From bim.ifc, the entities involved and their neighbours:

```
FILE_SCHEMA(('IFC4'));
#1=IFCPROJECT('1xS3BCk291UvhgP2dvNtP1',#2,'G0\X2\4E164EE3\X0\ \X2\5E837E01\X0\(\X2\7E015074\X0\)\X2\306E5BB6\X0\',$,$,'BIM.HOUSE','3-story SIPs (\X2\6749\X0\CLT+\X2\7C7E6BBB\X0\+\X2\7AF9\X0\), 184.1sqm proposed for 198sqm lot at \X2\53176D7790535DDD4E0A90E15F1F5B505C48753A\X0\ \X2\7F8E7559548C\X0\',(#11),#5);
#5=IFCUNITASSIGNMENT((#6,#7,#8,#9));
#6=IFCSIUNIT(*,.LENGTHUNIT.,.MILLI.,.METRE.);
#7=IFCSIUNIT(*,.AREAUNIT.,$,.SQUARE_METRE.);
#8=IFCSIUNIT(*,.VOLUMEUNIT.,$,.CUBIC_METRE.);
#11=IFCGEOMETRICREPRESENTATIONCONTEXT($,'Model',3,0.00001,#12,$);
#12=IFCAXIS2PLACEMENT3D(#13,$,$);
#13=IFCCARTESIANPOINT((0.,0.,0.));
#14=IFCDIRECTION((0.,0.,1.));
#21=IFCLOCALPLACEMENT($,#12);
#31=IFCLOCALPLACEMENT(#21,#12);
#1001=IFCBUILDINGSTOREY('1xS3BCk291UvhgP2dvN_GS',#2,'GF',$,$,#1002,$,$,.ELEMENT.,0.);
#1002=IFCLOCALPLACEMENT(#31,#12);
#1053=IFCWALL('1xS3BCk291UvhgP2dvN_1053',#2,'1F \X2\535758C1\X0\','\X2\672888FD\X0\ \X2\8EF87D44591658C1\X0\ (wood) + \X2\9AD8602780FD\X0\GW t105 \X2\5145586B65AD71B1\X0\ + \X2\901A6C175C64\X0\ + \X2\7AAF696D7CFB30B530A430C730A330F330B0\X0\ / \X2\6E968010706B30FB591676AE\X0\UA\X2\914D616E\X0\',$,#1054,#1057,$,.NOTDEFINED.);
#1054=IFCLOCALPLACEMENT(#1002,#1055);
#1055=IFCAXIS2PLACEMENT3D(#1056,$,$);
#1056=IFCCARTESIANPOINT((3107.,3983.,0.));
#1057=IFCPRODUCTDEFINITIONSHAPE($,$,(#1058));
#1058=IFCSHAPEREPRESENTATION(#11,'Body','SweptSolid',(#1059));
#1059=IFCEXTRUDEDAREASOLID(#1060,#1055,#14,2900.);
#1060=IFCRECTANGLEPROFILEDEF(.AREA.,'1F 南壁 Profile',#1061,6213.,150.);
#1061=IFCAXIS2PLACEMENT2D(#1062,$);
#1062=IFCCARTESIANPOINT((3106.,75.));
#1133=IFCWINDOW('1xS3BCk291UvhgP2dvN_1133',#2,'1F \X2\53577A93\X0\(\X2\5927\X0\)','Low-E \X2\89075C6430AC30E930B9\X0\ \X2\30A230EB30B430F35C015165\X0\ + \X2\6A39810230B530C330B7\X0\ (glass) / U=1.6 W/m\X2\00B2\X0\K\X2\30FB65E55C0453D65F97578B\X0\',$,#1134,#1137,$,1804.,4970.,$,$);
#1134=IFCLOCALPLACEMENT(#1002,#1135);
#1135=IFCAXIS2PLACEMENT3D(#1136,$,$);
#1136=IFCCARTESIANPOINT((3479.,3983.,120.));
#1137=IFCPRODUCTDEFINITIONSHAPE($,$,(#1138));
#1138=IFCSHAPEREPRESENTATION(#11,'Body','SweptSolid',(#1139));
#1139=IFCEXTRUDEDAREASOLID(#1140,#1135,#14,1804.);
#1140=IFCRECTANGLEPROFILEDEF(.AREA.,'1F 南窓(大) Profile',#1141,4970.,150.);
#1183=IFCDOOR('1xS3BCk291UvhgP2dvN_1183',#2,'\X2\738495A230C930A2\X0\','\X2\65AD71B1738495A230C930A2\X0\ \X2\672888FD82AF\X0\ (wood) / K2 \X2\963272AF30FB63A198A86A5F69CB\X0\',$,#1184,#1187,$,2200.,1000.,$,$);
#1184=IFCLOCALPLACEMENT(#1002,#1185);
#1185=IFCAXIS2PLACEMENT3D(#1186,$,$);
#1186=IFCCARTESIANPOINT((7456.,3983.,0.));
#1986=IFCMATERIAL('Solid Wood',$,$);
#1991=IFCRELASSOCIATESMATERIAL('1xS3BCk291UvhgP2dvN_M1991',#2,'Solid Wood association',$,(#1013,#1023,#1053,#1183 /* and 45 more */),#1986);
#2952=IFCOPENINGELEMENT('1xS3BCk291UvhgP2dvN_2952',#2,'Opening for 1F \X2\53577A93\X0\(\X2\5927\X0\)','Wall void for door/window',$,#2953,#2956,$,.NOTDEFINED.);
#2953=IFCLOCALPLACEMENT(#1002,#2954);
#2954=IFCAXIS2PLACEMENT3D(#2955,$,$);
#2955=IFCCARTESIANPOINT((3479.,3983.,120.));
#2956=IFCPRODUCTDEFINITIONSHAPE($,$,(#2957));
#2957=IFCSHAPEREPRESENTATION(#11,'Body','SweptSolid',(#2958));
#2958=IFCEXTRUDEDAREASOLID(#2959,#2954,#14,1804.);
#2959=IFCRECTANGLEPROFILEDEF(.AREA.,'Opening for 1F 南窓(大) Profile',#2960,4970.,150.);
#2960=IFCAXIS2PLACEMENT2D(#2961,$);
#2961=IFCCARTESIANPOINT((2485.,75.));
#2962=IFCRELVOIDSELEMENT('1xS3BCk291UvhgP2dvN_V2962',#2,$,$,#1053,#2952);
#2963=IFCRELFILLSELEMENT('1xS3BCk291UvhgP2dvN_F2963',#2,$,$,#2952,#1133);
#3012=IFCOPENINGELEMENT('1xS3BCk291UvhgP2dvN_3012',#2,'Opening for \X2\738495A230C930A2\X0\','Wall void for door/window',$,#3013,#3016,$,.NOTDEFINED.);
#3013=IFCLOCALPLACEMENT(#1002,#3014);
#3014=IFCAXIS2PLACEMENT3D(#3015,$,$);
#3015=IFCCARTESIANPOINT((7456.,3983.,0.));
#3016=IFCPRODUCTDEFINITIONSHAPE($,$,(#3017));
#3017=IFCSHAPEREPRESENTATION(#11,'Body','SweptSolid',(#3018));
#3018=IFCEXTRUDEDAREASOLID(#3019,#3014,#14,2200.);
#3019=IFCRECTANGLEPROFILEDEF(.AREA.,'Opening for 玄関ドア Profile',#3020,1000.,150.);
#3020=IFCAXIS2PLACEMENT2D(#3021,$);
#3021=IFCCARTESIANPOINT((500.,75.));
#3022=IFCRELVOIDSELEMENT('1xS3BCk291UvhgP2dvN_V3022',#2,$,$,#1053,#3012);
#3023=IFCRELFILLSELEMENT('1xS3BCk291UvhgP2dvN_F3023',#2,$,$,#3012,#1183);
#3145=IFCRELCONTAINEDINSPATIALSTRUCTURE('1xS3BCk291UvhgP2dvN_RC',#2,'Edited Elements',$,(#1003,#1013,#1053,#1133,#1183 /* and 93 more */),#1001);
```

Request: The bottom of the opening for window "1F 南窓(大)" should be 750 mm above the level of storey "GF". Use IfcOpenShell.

```python
import numpy as np
import ifcopenshell
import ifcopenshell.api.geometry
import ifcopenshell.geom
import ifcopenshell.util.element
import ifcopenshell.util.placement
import ifcopenshell.util.shape
import ifcopenshell.util.unit

model = ifcopenshell.open("bim.ifc")
unit_scale = ifcopenshell.util.unit.calculate_unit_scale(model)

window = model.by_id(1133)
opening = window.FillsVoids[0].RelatingOpeningElement
storey = ifcopenshell.util.element.get_container(window, ifc_class="IfcBuildingStorey")
level = ifcopenshell.util.placement.get_local_placement(storey.ObjectPlacement)[2, 3]

# The opening's origin need not be at the sill, so measure its lowest point.
shape = ifcopenshell.geom.create_shape(ifcopenshell.geom.settings(), opening)
bottom = ifcopenshell.util.shape.get_shape_bottom_elevation(shape, shape.geometry) / unit_scale
dz = level + 0.75 / unit_scale - bottom

shift = np.array([0.0, 0.0, dz])
# The window is not placed relative to its opening, so move both.
for product in (opening, window):
    matrix = ifcopenshell.util.placement.get_local_placement(product.ObjectPlacement)
    matrix[:3, 3] += shift
    ifcopenshell.api.geometry.edit_object_placement(model, product=product, matrix=matrix, is_si=False)

print(f"moved by {dz * unit_scale:+.3f} m")

model.write("bim_v2.ifc")
```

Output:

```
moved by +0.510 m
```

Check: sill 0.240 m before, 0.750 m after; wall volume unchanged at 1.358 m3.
